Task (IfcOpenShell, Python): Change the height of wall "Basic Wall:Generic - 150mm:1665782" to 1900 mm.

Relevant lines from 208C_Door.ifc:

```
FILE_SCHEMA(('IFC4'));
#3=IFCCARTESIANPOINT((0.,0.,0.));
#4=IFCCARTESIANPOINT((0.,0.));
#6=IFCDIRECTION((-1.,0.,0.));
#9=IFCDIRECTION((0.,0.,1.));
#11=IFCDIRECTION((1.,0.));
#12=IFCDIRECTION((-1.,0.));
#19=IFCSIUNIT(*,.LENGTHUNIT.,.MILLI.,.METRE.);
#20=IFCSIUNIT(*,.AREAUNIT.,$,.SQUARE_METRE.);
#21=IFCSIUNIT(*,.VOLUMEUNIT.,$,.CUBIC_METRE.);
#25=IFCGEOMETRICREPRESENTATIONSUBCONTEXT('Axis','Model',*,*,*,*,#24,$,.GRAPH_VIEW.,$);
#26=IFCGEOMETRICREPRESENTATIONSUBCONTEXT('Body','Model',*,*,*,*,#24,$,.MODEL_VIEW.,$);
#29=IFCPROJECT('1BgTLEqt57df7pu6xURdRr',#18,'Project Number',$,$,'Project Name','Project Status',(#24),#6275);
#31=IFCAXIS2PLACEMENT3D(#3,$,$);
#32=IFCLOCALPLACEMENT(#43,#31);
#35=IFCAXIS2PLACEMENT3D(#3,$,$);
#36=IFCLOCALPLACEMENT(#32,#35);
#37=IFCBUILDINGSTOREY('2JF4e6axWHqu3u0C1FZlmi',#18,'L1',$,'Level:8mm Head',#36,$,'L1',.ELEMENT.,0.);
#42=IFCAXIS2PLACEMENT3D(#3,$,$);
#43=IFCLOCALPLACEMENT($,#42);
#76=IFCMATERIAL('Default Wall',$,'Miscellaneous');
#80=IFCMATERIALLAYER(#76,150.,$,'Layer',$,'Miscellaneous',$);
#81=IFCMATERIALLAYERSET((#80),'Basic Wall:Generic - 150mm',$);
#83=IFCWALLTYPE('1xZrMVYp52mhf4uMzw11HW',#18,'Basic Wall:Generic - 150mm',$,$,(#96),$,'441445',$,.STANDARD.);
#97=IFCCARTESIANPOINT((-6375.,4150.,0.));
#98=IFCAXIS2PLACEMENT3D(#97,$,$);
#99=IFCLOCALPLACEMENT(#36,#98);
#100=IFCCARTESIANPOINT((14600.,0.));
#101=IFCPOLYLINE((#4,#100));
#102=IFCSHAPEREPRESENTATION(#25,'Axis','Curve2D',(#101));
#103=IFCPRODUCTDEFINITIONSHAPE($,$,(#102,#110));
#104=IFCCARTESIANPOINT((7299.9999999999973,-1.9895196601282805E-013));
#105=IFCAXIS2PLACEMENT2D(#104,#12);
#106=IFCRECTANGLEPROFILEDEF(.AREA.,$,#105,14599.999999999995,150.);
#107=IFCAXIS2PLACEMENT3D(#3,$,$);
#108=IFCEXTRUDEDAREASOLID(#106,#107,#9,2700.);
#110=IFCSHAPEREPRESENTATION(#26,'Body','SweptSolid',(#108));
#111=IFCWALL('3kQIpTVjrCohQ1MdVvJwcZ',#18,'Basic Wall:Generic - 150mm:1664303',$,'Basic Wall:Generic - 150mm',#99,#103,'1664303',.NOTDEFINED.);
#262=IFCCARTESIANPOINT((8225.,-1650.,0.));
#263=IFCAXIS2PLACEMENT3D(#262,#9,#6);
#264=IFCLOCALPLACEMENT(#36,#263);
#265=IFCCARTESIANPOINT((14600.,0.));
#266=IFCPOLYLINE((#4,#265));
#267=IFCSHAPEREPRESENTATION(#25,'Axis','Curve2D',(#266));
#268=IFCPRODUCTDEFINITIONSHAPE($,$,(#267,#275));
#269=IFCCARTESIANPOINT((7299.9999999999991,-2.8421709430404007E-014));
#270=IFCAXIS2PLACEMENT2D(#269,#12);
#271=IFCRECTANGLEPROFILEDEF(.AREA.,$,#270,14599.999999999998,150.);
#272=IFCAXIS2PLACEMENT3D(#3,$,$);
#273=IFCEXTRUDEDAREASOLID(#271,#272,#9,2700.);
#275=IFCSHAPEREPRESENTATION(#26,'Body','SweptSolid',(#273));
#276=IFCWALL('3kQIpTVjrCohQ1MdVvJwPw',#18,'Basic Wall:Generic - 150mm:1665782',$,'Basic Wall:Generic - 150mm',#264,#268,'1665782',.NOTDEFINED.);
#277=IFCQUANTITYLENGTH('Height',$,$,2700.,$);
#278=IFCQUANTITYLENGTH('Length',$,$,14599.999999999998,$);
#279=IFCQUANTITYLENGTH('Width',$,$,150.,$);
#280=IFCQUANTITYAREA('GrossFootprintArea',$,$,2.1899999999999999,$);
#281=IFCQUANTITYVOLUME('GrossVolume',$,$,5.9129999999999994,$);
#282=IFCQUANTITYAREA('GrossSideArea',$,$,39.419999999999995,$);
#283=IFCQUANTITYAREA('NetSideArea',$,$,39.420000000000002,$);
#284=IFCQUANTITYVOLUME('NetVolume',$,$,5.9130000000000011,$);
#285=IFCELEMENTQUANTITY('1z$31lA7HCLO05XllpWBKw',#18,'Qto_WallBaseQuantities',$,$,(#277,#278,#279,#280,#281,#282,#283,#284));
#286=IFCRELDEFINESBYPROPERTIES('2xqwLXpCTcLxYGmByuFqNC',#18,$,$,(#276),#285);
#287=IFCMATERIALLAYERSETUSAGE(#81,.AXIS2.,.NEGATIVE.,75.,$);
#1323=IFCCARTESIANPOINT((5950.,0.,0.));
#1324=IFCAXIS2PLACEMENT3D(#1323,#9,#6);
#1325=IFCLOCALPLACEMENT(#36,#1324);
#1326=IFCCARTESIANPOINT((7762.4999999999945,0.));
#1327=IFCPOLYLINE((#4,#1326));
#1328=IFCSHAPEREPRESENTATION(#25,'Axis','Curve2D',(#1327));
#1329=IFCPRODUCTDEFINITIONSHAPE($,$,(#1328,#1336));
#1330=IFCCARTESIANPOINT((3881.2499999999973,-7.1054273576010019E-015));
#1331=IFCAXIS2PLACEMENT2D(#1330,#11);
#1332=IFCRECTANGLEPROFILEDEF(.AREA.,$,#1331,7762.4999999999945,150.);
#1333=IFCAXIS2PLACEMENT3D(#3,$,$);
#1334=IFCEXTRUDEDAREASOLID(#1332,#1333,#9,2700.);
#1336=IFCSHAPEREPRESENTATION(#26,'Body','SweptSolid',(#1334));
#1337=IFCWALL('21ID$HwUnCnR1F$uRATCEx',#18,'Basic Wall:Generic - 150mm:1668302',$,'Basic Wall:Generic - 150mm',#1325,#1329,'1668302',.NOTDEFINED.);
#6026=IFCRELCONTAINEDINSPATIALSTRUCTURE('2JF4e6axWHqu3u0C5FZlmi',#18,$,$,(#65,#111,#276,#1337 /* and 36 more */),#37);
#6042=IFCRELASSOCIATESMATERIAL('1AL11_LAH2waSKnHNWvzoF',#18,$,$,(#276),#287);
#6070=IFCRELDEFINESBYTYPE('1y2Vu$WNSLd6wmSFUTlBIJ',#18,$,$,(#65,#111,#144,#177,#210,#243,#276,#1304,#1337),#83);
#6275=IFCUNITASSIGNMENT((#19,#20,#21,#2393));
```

```python
import ifcopenshell
import ifcopenshell.api.pset
import ifcopenshell.geom
import ifcopenshell.util.element
import ifcopenshell.util.representation
import ifcopenshell.util.shape
import ifcopenshell.util.unit

model = ifcopenshell.open("208C_Door.ifc")
unit_scale = ifcopenshell.util.unit.calculate_unit_scale(model)
area_scale = ifcopenshell.util.unit.calculate_unit_scale(model, "AREAUNIT")
volume_scale = ifcopenshell.util.unit.calculate_unit_scale(model, "VOLUMEUNIT")
settings = ifcopenshell.geom.settings()


def volume(element):
    """Net volume in cubic metres, openings subtracted."""
    shape = ifcopenshell.geom.create_shape(settings, element)
    return ifcopenshell.util.shape.get_volume(shape.geometry)


wall = model.by_guid("3kQIpTVjrCohQ1MdVvJwPw")
before = volume(wall)

body = ifcopenshell.util.representation.get_representation(wall, "Model", "Body")
solid = body.Items[0]
old_height = solid.Depth
solid.Depth = 1900.0
after = volume(wall)
thickness = 0.15  # wall thickness in metres

# Update the stored height, areas and volumes.
qto = model.by_id(ifcopenshell.util.element.get_pset(wall, "Qto_WallBaseQuantities", should_inherit=False)["id"])
ifcopenshell.api.pset.edit_qto(model, qto=qto, properties={
    "Height": solid.Depth,
    "GrossVolume": ifcopenshell.util.element.get_pset(wall, "Qto_WallBaseQuantities", "GrossVolume") * solid.Depth / old_height,
    "GrossSideArea": ifcopenshell.util.element.get_pset(wall, "Qto_WallBaseQuantities", "GrossSideArea") * solid.Depth / old_height,
    "NetSideArea": after / thickness / area_scale,
    "NetVolume": after / volume_scale,
})

print(f"height {old_height:g} -> {solid.Depth:g}, volume {before:.3f} -> {after:.3f} m3")

model.write("208C_Door_updated.ifc")
```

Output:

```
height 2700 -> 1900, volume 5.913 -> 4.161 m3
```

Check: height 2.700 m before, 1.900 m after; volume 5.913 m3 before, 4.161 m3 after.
